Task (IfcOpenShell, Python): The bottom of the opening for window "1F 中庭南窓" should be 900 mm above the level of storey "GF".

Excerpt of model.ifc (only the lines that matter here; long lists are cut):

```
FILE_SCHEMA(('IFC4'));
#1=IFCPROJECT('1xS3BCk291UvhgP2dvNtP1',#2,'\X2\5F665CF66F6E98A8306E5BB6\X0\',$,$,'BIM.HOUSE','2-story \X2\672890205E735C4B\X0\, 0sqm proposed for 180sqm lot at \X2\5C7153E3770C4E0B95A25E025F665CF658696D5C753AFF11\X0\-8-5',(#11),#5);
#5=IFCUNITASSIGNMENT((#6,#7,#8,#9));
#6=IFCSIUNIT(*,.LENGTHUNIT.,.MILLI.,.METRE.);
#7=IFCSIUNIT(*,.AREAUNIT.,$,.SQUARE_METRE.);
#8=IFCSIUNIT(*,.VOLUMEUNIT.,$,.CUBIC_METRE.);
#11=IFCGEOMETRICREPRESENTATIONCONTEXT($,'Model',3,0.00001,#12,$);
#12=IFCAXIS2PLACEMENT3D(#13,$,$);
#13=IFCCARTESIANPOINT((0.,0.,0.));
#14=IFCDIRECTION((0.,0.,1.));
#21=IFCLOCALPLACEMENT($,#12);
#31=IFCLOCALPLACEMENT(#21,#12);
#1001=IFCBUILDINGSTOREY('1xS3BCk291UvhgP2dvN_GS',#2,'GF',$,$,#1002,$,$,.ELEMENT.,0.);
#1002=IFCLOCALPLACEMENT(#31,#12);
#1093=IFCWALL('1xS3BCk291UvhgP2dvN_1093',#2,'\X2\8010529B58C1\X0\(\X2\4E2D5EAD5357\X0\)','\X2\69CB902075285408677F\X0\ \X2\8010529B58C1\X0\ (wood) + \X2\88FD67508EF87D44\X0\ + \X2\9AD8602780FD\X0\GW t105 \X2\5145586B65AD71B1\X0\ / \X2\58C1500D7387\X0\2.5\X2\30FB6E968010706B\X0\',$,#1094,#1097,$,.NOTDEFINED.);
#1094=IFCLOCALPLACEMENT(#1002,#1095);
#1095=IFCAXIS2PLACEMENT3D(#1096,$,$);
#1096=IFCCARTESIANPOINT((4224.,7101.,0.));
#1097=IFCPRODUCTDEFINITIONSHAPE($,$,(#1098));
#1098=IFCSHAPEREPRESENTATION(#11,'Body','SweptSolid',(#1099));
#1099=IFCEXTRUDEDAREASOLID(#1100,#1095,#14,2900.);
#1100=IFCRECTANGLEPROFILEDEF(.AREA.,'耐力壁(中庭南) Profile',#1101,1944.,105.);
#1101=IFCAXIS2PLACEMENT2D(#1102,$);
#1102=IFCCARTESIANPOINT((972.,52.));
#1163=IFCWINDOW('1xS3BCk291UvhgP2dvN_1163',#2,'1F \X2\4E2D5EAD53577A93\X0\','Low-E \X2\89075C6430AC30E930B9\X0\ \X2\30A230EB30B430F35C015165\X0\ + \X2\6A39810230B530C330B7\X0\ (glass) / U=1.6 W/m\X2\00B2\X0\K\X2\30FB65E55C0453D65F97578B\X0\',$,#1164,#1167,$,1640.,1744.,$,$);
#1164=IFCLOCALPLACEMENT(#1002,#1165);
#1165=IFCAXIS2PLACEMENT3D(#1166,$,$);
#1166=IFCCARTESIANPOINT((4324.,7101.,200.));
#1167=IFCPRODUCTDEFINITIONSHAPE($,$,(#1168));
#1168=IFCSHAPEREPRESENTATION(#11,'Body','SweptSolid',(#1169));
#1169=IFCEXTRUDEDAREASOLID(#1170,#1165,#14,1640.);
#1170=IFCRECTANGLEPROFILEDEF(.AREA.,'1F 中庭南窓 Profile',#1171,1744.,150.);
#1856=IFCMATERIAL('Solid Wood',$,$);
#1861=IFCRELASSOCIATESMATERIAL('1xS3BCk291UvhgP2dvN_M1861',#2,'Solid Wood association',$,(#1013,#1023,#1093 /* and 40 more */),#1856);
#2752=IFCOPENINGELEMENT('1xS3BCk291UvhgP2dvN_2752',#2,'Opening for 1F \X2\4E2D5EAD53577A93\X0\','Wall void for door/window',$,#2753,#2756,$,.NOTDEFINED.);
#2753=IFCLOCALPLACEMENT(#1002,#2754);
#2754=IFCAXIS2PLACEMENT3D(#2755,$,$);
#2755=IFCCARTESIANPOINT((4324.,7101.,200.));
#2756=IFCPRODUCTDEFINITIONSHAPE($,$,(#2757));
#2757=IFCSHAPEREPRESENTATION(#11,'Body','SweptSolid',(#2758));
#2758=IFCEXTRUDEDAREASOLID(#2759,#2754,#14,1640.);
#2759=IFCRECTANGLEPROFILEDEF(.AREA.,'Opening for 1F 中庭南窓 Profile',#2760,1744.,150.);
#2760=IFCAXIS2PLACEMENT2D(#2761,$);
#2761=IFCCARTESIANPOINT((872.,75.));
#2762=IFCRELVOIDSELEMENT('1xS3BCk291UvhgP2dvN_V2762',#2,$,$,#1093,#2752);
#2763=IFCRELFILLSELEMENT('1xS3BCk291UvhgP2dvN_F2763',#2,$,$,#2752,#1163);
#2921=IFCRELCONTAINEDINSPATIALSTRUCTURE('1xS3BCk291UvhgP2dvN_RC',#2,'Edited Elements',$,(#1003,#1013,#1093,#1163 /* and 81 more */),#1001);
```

```python
import numpy as np
import ifcopenshell
import ifcopenshell.api.geometry
import ifcopenshell.geom
import ifcopenshell.util.element
import ifcopenshell.util.placement
import ifcopenshell.util.shape
import ifcopenshell.util.unit

model = ifcopenshell.open("model.ifc")
unit_scale = ifcopenshell.util.unit.calculate_unit_scale(model)

window = model.by_guid("1xS3BCk291UvhgP2dvN_1163")
opening = window.FillsVoids[0].RelatingOpeningElement
storey = ifcopenshell.util.element.get_container(window, ifc_class="IfcBuildingStorey")
level = ifcopenshell.util.placement.get_local_placement(storey.ObjectPlacement)[2, 3]

# The opening's origin need not be at the sill, so measure its lowest point.
shape = ifcopenshell.geom.create_shape(ifcopenshell.geom.settings(), opening)
bottom = ifcopenshell.util.shape.get_shape_bottom_elevation(shape, shape.geometry) / unit_scale
dz = level + 900.0 - bottom

shift = np.array([0.0, 0.0, dz])
# The window is not placed relative to its opening, so move both.
for product in (opening, window):
    matrix = ifcopenshell.util.placement.get_local_placement(product.ObjectPlacement)
    matrix[:3, 3] += shift
    ifcopenshell.api.geometry.edit_object_placement(model, product=product, matrix=matrix, is_si=False)

print(f"moved by {dz * unit_scale:+.3f} m")

model.write("model_rev.ifc")
```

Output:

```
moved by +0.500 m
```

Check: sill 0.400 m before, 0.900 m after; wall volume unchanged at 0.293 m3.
